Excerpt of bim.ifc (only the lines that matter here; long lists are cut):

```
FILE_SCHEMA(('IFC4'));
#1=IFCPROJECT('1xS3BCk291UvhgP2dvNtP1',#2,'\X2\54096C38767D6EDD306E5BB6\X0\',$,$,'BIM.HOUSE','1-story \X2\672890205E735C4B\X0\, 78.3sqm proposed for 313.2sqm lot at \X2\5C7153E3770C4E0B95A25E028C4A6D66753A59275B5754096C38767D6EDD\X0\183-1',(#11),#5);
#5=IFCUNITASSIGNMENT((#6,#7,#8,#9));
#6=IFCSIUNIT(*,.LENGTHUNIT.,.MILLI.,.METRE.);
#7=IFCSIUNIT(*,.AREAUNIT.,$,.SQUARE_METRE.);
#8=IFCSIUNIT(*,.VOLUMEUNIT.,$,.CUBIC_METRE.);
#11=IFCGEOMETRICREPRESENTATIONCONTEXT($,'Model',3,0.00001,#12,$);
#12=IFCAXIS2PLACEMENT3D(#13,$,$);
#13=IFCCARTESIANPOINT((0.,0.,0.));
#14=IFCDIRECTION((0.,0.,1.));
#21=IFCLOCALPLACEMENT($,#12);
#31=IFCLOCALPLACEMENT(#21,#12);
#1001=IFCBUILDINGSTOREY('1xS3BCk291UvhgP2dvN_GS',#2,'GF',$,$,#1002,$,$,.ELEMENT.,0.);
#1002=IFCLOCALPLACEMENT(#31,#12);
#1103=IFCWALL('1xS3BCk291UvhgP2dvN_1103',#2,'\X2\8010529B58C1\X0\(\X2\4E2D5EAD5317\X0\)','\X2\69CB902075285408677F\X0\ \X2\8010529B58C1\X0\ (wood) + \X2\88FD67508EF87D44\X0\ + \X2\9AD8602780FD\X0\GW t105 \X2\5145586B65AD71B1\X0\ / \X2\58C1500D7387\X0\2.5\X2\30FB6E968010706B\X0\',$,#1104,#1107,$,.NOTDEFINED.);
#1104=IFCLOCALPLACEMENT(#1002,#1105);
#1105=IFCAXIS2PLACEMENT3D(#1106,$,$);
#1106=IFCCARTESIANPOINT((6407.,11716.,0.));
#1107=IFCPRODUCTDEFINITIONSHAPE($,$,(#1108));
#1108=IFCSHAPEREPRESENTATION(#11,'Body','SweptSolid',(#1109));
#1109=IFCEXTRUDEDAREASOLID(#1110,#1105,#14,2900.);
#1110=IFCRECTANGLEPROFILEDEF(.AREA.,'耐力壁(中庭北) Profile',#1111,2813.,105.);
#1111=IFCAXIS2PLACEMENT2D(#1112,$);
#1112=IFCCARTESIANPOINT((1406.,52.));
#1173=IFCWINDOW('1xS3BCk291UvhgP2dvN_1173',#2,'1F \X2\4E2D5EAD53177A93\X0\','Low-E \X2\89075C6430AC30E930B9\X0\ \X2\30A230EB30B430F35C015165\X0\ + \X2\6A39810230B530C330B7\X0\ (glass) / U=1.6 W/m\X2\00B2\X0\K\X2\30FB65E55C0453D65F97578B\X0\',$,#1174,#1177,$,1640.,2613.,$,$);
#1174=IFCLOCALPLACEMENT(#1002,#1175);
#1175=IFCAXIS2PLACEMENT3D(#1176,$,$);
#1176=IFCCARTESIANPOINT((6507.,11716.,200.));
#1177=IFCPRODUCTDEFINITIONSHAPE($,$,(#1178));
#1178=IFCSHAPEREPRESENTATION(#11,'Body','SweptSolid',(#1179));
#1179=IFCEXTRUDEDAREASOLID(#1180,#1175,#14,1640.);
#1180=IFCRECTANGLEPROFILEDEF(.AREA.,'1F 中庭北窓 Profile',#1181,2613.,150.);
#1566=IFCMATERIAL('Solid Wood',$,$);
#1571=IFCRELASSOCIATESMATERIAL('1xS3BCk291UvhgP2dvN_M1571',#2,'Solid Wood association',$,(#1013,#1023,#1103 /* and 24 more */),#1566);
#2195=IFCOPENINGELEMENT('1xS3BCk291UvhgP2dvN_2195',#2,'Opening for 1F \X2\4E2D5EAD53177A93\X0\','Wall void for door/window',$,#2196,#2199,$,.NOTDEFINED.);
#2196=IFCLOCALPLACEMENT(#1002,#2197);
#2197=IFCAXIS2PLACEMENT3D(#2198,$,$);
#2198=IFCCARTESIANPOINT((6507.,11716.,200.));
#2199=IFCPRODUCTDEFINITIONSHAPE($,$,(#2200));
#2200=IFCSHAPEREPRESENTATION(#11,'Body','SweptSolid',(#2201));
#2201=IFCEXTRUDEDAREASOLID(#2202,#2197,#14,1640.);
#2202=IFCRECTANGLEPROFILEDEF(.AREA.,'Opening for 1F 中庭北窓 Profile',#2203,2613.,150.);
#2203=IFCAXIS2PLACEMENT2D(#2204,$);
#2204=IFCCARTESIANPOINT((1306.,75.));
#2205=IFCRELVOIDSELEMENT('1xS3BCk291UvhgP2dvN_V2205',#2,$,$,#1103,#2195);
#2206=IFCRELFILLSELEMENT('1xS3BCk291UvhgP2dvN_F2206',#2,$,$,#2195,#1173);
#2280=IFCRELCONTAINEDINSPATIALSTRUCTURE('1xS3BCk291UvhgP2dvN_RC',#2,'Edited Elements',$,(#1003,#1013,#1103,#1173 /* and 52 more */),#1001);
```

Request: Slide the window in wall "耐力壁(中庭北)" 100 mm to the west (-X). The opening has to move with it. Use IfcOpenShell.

```python
import ifcopenshell
import ifcopenshell.api.geometry
import ifcopenshell.util.placement
import ifcopenshell.util.unit

model = ifcopenshell.open("bim.ifc")
unit_scale = ifcopenshell.util.unit.calculate_unit_scale(model)

window = model.by_id(1173)
opening = window.FillsVoids[0].RelatingOpeningElement
wall = opening.VoidsElements[0].RelatingBuildingElement

wall_matrix = ifcopenshell.util.placement.get_local_placement(wall.ObjectPlacement)
shift = wall_matrix[:3, 0] * -0.1 / unit_scale
before = ifcopenshell.util.placement.get_local_placement(window.ObjectPlacement)[:3, 3].copy()

# The window is not placed relative to its opening, so move both.
for product in (opening, window):
    matrix = ifcopenshell.util.placement.get_local_placement(product.ObjectPlacement)
    matrix[:3, 3] += shift
    ifcopenshell.api.geometry.edit_object_placement(model, product=product, matrix=matrix, is_si=False)

after = ifcopenshell.util.placement.get_local_placement(window.ObjectPlacement)[:3, 3]
print("window moved by", (after - before).round(3) + 0.0)

model.write("bim_edited.ifc")
```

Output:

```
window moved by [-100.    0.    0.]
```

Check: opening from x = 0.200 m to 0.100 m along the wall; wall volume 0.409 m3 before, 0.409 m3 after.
